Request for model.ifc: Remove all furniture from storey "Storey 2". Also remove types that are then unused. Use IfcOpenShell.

First a look at what the model holds.

```python
import ifcopenshell
import ifcopenshell.util.element

model = ifcopenshell.open("model.ifc")
print(model.schema)
storey = next(s for s in model.by_type("IfcBuildingStorey") if s.Name == "Storey 2")
furniture = [e for e in ifcopenshell.util.element.get_decomposition(storey) if e.is_a("IfcFurnishingElement")]
seen = {}
for e in furniture:
    element_type = ifcopenshell.util.element.get_type(e)
    name = element_type.Name if element_type not in (None, e) else None
    seen[name] = seen.get(name, 0) + 1
for name, count in sorted(seen.items(), key=str):
    print(count, "x", name)
```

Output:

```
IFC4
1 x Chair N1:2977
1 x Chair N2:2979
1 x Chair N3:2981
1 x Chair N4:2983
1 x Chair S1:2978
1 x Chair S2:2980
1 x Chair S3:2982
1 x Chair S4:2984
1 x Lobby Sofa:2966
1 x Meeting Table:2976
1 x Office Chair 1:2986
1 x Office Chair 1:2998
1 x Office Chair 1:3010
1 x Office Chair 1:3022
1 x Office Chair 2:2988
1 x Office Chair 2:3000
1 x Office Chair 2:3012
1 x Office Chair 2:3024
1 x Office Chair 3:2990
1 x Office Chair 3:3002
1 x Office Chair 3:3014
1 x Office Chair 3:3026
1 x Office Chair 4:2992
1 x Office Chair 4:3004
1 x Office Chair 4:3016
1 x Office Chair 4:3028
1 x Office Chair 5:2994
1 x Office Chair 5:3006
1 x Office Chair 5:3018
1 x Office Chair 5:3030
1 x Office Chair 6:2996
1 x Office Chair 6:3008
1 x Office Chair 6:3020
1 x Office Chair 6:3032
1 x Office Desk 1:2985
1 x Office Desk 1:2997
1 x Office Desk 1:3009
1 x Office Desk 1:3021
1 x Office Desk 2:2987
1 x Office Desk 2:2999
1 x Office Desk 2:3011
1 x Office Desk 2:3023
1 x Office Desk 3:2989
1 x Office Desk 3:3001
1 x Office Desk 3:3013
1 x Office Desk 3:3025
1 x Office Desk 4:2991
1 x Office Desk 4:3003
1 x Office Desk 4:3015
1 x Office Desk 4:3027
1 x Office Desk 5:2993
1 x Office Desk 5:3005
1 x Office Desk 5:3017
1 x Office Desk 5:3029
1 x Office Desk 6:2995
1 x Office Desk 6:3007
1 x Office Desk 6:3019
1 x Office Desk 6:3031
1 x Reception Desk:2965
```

```python
import ifcopenshell
import ifcopenshell.api.root
import ifcopenshell.util.element

model = ifcopenshell.open("model.ifc")

storey = next(s for s in model.by_type("IfcBuildingStorey") if s.Name == "Storey 2")
furniture = [e for e in ifcopenshell.util.element.get_decomposition(storey) if e.is_a("IfcFurnishingElement")]
types = {ifcopenshell.util.element.get_type(e) for e in furniture} - {None, *furniture}

for e in furniture:
    ifcopenshell.api.root.remove_product(model, product=e)
print(len(furniture), "removed")

unused = [t for t in types if not ifcopenshell.util.element.get_types(t)]
for t in unused:
    ifcopenshell.api.root.remove_product(model, product=t)
print(len(unused), "unused types removed")

model.write("model_updated.ifc")
```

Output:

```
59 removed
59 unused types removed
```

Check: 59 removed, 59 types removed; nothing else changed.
